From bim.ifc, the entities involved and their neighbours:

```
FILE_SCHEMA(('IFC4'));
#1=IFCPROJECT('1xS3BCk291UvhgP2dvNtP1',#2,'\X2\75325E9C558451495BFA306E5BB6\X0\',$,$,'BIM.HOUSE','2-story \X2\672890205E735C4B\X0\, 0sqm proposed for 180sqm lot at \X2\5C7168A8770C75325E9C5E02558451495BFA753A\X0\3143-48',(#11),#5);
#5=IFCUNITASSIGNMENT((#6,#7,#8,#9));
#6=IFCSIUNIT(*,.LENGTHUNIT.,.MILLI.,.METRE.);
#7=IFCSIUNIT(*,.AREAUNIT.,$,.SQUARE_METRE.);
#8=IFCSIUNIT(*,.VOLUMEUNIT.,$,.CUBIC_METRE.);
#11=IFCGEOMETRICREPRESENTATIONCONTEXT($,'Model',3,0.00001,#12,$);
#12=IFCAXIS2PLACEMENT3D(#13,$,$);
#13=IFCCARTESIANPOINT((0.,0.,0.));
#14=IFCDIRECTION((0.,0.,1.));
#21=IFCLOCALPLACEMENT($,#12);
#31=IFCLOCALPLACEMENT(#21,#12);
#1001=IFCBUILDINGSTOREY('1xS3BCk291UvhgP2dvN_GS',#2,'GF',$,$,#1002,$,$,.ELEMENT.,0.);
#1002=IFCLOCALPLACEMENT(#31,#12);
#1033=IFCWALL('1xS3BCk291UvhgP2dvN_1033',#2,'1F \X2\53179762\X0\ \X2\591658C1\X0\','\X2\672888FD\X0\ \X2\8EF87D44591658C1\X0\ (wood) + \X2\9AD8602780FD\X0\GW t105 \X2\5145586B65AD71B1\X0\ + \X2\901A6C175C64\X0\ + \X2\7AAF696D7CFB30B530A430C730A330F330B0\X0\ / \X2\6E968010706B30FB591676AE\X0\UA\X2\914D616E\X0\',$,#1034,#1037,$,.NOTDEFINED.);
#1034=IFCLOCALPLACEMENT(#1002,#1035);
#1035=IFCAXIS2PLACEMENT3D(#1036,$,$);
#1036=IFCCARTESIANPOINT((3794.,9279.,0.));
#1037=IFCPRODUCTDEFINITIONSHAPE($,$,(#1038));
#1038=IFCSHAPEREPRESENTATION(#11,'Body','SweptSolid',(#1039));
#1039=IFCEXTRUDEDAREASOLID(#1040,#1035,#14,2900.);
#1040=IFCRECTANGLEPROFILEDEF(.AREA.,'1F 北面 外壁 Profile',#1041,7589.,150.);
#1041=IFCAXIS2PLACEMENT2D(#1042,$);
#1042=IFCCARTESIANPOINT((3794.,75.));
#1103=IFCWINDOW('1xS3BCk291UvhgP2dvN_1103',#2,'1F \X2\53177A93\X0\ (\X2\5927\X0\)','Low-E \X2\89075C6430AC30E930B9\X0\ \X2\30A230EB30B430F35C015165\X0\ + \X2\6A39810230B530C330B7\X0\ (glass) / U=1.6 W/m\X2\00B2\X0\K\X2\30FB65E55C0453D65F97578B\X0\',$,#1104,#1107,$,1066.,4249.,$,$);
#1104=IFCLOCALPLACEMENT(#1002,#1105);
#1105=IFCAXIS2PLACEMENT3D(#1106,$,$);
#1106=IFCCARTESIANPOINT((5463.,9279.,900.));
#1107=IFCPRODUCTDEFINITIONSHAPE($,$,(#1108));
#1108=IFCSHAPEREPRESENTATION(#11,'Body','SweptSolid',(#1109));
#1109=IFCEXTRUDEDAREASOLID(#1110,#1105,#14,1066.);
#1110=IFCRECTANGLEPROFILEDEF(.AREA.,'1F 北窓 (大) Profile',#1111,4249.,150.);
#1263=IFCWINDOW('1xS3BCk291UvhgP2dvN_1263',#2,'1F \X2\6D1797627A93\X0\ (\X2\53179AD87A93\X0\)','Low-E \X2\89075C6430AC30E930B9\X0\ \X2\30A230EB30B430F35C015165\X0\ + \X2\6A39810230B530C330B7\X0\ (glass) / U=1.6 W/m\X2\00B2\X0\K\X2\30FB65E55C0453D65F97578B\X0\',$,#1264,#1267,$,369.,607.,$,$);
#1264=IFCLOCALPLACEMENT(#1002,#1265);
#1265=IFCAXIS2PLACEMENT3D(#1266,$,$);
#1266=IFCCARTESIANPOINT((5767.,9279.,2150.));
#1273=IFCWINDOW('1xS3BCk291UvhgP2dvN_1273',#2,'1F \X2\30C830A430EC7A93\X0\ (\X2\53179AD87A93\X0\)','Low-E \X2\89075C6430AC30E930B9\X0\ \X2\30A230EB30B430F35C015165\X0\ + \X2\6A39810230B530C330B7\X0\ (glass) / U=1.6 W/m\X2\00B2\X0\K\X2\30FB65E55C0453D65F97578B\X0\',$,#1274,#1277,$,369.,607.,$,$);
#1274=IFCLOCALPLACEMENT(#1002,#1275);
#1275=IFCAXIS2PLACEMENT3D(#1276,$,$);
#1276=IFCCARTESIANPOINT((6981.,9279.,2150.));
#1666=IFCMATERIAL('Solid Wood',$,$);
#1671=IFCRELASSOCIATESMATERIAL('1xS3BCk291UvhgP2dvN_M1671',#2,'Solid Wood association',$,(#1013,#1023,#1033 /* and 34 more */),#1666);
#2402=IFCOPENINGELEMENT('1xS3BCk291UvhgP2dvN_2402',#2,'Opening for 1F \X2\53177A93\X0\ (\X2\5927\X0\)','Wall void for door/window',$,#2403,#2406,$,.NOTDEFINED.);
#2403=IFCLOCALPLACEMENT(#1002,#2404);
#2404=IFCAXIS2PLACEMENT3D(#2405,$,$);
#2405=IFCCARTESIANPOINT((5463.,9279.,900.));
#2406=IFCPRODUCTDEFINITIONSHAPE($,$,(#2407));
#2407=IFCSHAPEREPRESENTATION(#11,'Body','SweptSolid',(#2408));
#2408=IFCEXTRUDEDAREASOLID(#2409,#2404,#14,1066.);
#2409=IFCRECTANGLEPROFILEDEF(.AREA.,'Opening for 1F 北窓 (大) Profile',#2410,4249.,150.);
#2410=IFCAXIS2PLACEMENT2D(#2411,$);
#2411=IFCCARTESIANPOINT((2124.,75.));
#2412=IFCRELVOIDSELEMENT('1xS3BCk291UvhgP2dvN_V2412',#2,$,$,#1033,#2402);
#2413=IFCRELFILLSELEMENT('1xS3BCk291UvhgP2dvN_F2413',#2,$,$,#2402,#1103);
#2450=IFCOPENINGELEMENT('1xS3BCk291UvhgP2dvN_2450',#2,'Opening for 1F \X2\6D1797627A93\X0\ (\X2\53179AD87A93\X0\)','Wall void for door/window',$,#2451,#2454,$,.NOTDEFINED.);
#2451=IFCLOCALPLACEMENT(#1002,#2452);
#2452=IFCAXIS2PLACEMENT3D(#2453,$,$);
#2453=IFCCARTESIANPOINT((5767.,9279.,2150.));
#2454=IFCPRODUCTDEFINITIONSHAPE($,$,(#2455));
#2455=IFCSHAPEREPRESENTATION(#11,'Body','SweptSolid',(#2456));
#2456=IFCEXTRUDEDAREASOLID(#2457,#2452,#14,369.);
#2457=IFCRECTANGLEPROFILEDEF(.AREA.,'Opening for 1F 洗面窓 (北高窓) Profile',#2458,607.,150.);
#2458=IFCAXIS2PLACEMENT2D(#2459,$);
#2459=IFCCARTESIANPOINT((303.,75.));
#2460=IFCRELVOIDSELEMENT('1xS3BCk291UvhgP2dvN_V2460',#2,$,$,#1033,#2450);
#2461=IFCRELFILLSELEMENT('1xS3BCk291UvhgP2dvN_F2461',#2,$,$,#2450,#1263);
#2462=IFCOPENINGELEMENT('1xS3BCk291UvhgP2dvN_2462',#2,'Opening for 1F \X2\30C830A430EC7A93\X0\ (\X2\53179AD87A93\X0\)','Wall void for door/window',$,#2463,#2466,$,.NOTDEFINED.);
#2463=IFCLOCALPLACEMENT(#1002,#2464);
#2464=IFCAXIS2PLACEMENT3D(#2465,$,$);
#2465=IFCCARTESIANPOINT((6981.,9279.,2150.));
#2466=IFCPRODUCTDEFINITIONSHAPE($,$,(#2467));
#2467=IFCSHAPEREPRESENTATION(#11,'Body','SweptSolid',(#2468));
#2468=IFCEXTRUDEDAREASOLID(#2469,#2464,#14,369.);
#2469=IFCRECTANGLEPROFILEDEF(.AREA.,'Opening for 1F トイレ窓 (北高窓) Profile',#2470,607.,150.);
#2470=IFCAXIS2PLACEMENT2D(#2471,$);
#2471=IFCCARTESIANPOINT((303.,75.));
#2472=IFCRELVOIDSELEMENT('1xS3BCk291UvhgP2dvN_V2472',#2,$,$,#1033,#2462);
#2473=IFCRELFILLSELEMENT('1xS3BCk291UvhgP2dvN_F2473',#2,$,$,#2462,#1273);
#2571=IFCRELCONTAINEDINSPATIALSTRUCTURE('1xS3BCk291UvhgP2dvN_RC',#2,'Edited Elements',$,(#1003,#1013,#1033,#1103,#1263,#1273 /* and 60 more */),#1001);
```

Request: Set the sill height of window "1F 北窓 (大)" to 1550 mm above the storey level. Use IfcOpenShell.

```python
import numpy as np
import ifcopenshell
import ifcopenshell.api.geometry
import ifcopenshell.geom
import ifcopenshell.util.element
import ifcopenshell.util.placement
import ifcopenshell.util.shape
import ifcopenshell.util.unit

model = ifcopenshell.open("bim.ifc")
unit_scale = ifcopenshell.util.unit.calculate_unit_scale(model)

window = model.by_guid("1xS3BCk291UvhgP2dvN_1103")
opening = window.FillsVoids[0].RelatingOpeningElement
storey = ifcopenshell.util.element.get_container(window, ifc_class="IfcBuildingStorey")
level = ifcopenshell.util.placement.get_local_placement(storey.ObjectPlacement)[2, 3]

# The opening's origin need not be at the sill, so measure its lowest point.
shape = ifcopenshell.geom.create_shape(ifcopenshell.geom.settings(), opening)
bottom = ifcopenshell.util.shape.get_shape_bottom_elevation(shape, shape.geometry) / unit_scale
dz = level + 1.55 / unit_scale - bottom

shift = np.array([0.0, 0.0, dz])
# The window is not placed relative to its opening, so move both.
for product in (opening, window):
    matrix = ifcopenshell.util.placement.get_local_placement(product.ObjectPlacement)
    matrix[:3, 3] += shift
    ifcopenshell.api.geometry.edit_object_placement(model, product=product, matrix=matrix, is_si=False)

print(f"moved by {dz * unit_scale:+.3f} m")

model.write("bim_updated.ifc")
```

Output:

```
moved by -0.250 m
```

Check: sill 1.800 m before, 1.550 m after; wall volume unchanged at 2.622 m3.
